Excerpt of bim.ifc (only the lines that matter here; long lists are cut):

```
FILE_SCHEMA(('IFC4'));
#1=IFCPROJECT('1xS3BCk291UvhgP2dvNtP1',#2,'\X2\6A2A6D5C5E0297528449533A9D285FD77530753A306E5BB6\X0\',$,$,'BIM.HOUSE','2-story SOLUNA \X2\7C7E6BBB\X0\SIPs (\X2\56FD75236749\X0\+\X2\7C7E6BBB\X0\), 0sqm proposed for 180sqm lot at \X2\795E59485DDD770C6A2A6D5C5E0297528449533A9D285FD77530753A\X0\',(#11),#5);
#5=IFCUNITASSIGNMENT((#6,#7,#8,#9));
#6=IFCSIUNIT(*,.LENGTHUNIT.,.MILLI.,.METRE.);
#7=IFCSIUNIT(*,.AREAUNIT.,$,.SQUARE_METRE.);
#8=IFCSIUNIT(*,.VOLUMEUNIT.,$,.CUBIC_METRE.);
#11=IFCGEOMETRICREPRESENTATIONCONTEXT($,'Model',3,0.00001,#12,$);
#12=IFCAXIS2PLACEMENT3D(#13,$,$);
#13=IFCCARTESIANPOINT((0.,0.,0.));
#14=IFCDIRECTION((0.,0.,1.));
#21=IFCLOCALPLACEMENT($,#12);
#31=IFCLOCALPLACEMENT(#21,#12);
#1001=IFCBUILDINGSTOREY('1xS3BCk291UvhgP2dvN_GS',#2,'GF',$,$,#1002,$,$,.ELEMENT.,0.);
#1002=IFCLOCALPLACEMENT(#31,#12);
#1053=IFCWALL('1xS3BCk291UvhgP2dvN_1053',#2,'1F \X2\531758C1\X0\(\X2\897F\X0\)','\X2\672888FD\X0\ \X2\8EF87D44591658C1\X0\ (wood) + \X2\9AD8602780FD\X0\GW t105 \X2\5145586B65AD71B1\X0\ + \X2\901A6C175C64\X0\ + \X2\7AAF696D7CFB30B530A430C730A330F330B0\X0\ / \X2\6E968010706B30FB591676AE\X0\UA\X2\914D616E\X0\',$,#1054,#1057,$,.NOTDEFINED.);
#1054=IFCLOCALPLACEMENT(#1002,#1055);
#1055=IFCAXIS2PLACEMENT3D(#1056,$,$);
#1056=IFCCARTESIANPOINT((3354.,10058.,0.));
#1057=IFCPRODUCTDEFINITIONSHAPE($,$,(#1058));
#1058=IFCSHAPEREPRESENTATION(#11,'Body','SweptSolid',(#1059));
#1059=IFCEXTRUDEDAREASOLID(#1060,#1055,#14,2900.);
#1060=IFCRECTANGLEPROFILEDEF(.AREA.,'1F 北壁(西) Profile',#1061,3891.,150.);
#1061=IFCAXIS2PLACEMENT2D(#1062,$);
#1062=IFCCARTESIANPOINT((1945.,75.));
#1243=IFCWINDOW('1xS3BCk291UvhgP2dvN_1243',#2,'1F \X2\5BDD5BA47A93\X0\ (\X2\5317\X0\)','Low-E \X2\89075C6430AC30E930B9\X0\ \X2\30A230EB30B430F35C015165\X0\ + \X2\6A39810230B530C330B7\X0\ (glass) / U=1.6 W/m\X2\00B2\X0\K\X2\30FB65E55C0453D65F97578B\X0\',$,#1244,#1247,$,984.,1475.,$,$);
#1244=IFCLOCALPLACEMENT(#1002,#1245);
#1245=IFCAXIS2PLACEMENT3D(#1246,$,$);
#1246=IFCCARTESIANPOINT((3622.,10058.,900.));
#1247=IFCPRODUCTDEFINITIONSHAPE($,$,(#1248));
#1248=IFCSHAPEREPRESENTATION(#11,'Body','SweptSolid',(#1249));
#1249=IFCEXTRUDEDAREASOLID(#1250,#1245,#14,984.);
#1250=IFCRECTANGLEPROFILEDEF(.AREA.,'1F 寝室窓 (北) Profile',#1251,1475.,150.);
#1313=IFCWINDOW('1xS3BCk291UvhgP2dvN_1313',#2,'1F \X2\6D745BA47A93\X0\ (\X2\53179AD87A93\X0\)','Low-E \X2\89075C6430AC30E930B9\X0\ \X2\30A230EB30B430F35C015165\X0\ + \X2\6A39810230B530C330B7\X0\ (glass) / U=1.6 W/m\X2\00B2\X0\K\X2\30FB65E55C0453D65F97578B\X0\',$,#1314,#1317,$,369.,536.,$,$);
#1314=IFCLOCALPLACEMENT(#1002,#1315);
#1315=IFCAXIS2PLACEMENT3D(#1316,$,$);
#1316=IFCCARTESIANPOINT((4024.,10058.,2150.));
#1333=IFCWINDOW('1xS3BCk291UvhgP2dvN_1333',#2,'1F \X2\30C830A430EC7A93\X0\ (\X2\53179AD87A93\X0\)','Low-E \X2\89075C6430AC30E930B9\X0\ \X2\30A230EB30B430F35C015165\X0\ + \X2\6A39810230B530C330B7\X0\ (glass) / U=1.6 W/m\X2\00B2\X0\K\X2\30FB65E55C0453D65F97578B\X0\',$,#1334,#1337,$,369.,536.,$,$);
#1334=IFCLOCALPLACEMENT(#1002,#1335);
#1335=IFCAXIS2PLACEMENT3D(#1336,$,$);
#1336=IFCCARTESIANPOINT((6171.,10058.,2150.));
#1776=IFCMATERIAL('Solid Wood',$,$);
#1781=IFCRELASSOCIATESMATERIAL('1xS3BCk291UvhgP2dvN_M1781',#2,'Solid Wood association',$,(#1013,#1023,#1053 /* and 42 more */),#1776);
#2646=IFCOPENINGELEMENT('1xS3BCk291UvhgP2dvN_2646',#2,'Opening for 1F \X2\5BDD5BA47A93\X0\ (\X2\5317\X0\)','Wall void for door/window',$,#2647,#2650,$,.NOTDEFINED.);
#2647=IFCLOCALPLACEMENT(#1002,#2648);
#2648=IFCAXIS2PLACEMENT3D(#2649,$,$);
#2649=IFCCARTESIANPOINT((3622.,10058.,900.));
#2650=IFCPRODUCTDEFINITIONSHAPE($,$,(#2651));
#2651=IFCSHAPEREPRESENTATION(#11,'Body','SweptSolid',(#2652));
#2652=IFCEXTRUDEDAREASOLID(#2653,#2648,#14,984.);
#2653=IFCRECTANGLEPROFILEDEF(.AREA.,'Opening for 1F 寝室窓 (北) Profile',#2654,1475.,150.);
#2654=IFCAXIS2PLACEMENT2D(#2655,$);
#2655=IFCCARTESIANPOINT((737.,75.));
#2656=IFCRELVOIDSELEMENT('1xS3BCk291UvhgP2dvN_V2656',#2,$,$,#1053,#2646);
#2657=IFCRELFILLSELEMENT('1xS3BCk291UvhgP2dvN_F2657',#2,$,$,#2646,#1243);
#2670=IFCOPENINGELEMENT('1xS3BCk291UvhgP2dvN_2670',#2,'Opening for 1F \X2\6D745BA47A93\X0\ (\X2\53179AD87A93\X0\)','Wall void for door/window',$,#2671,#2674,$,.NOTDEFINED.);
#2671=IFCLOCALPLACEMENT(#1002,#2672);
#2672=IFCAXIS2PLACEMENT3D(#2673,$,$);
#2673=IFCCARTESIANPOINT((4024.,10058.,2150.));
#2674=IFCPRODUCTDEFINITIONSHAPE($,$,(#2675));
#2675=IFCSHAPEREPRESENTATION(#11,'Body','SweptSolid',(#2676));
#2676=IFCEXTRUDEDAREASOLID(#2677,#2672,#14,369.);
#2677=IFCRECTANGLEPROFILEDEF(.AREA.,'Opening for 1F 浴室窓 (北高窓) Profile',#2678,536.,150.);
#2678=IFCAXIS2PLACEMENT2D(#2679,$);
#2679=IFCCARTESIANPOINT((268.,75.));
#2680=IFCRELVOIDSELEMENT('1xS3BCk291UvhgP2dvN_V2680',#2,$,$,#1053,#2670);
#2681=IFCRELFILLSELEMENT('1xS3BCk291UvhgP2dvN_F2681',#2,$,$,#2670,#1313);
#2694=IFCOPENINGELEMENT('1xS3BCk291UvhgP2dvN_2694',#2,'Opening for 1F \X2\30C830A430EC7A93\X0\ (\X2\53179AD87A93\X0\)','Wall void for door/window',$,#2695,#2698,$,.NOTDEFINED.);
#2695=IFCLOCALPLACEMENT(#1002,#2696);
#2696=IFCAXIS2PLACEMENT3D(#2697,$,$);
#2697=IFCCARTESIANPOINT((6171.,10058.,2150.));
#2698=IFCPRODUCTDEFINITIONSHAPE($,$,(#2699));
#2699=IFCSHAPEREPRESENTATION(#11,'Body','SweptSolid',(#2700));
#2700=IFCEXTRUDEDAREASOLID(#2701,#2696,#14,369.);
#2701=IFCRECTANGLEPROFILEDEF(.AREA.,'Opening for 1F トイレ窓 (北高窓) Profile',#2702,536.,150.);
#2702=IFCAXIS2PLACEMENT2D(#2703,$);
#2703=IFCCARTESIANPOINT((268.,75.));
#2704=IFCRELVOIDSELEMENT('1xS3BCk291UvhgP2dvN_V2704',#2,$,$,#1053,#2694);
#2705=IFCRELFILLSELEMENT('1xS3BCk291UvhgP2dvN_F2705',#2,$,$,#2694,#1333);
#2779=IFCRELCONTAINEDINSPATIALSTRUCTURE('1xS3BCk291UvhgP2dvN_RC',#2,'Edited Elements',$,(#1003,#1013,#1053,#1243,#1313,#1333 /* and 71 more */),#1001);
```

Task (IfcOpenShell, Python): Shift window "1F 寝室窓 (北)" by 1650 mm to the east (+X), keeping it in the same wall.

```python
import ifcopenshell
import ifcopenshell.api.geometry
import ifcopenshell.util.placement

model = ifcopenshell.open("bim.ifc")

window = model.by_id(1243)
opening = window.FillsVoids[0].RelatingOpeningElement
wall = opening.VoidsElements[0].RelatingBuildingElement

wall_matrix = ifcopenshell.util.placement.get_local_placement(wall.ObjectPlacement)
shift = wall_matrix[:3, 0] * 1650.0
before = ifcopenshell.util.placement.get_local_placement(window.ObjectPlacement)[:3, 3].copy()

# The window is not placed relative to its opening, so move both.
for product in (opening, window):
    matrix = ifcopenshell.util.placement.get_local_placement(product.ObjectPlacement)
    matrix[:3, 3] += shift
    ifcopenshell.api.geometry.edit_object_placement(model, product=product, matrix=matrix, is_si=False)

after = ifcopenshell.util.placement.get_local_placement(window.ObjectPlacement)[:3, 3]
print("window moved by", (after - before).round(3) + 0.0)

model.write("bim_updated.ifc")
```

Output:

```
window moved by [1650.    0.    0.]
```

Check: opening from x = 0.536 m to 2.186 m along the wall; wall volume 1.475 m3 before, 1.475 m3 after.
